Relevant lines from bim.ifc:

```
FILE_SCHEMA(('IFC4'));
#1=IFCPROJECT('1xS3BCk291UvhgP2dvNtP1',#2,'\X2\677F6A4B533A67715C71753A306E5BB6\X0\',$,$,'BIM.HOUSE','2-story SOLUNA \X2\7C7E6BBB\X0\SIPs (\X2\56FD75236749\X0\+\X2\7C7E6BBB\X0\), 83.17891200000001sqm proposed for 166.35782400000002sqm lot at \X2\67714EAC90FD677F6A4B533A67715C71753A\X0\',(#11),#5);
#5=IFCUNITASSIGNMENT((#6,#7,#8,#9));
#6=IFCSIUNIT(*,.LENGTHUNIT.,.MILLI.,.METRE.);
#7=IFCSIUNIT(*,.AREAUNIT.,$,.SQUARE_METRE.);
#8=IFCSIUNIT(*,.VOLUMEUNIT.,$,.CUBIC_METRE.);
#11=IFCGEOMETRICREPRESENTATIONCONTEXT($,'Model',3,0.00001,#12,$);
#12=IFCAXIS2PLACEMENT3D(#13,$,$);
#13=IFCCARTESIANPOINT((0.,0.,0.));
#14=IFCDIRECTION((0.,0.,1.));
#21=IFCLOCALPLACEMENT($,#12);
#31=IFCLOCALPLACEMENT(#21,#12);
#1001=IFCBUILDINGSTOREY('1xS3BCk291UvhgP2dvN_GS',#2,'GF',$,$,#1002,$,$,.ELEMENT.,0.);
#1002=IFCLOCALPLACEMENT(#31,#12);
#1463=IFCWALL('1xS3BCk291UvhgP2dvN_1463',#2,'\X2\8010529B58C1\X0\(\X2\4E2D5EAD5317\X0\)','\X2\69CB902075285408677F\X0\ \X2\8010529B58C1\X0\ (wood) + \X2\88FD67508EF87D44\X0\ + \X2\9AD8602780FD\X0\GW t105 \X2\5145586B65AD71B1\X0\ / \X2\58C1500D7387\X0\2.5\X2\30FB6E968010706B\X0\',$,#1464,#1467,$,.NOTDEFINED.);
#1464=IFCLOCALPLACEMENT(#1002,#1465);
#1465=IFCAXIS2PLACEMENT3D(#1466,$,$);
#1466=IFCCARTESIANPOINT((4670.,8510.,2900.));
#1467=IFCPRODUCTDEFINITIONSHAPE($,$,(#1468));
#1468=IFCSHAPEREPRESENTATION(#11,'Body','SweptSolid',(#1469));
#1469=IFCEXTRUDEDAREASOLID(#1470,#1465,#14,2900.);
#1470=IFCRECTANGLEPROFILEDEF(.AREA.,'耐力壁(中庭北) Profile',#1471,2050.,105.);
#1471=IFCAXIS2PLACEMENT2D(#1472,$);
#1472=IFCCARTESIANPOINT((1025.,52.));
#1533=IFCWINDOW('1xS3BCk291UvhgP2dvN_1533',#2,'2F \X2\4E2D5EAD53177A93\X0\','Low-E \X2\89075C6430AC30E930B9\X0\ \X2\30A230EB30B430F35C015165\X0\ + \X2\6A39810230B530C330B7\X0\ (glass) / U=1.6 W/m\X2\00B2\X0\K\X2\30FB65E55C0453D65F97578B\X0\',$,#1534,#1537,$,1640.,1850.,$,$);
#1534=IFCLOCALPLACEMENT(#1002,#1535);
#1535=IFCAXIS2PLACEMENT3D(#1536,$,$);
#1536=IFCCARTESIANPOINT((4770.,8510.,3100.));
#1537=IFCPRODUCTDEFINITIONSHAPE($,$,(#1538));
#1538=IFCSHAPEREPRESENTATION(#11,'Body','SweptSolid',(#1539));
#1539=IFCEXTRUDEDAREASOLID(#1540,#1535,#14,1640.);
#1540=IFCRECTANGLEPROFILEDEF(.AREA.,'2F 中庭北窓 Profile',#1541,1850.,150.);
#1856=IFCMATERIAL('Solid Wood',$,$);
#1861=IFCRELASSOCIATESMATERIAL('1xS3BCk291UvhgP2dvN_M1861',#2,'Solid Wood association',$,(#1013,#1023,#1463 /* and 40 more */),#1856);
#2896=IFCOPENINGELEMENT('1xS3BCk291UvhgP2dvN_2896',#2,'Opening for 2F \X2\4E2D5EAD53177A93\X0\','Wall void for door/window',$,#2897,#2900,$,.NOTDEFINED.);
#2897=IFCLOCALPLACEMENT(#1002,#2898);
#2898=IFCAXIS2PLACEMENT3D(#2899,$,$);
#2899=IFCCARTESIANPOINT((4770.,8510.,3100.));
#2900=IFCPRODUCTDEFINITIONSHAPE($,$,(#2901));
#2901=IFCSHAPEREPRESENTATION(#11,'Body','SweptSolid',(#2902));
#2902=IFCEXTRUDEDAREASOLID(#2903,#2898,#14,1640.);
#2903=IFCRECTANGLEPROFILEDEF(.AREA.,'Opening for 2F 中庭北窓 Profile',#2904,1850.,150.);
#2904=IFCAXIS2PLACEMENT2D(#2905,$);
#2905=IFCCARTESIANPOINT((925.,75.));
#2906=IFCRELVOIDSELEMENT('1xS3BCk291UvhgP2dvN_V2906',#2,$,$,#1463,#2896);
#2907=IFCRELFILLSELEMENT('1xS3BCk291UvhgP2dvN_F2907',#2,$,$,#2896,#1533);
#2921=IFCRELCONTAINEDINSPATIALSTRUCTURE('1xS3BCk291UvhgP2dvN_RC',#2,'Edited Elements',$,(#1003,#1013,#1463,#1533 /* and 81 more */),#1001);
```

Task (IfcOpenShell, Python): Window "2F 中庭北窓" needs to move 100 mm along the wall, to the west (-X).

```python
import ifcopenshell
import ifcopenshell.api.geometry
import ifcopenshell.util.placement
import ifcopenshell.util.unit

model = ifcopenshell.open("bim.ifc")
unit_scale = ifcopenshell.util.unit.calculate_unit_scale(model)

window = model.by_guid("1xS3BCk291UvhgP2dvN_1533")
opening = window.FillsVoids[0].RelatingOpeningElement
wall = opening.VoidsElements[0].RelatingBuildingElement

wall_matrix = ifcopenshell.util.placement.get_local_placement(wall.ObjectPlacement)
shift = wall_matrix[:3, 0] * -0.1 / unit_scale
before = ifcopenshell.util.placement.get_local_placement(window.ObjectPlacement)[:3, 3].copy()

# The window is not placed relative to its opening, so move both.
for product in (opening, window):
    matrix = ifcopenshell.util.placement.get_local_placement(product.ObjectPlacement)
    matrix[:3, 3] += shift
    ifcopenshell.api.geometry.edit_object_placement(model, product=product, matrix=matrix, is_si=False)

after = ifcopenshell.util.placement.get_local_placement(window.ObjectPlacement)[:3, 3]
print("window moved by", (after - before).round(3) + 0.0)

model.write("bim_updated.ifc")
```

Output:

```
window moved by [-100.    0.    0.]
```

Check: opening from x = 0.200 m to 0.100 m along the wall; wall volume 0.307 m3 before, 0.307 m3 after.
